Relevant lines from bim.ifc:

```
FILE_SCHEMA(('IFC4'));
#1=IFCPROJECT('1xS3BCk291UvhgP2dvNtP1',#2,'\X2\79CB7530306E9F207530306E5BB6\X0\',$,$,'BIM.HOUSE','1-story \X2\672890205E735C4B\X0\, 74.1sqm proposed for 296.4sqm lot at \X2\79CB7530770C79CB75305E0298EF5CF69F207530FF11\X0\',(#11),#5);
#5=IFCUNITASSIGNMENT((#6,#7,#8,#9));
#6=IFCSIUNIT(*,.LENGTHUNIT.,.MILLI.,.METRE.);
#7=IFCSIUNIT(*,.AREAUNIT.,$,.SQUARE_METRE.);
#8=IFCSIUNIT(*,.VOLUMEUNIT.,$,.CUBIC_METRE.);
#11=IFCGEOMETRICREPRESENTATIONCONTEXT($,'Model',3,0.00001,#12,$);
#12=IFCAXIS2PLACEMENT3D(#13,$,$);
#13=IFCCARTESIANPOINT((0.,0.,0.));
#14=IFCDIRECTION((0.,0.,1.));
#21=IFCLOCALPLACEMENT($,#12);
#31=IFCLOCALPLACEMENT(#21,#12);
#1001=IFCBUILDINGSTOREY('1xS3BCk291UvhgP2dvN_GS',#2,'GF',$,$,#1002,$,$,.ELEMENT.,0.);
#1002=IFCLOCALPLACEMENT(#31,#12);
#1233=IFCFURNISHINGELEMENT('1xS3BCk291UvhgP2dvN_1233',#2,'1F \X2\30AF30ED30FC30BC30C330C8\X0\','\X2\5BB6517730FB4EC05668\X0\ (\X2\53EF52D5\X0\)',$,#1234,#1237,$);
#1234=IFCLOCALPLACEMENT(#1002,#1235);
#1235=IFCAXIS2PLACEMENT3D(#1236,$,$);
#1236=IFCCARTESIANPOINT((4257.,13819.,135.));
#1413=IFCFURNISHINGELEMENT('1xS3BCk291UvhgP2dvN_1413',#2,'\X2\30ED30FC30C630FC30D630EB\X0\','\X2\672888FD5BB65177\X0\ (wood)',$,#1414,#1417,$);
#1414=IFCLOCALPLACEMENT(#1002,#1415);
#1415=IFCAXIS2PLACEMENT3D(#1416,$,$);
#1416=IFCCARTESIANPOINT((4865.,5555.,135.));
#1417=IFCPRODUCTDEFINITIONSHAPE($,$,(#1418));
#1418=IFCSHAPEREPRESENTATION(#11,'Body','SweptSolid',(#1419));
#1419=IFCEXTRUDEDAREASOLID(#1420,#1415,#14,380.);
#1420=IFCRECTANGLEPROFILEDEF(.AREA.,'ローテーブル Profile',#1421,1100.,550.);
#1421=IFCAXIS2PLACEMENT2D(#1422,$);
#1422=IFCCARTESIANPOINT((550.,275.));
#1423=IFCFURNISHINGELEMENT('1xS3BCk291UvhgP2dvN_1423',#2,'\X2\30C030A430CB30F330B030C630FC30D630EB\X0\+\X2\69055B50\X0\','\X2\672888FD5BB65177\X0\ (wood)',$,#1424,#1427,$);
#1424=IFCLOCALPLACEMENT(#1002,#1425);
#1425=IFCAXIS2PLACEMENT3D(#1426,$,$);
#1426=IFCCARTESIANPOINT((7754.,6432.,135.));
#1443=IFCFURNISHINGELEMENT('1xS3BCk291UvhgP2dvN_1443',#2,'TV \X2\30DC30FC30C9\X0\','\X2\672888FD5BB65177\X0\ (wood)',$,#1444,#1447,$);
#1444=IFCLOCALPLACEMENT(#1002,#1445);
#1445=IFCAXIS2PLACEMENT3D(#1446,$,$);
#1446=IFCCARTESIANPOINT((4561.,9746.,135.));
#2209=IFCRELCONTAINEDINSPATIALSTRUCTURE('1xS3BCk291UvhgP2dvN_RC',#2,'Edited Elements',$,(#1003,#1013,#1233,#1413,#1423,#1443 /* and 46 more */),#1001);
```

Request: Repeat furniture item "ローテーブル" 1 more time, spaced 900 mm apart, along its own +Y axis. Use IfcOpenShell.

```python
import ifcopenshell
import ifcopenshell.api.geometry
import ifcopenshell.api.root
import ifcopenshell.util.element
import ifcopenshell.util.placement
import ifcopenshell.util.unit

model = ifcopenshell.open("bim.ifc")
unit_scale = ifcopenshell.util.unit.calculate_unit_scale(model)


def reuse_history(source, copy):
    """copy_class also copies each property set's owner history, people and application; keep the originals."""
    for rel in copy.IsDefinedBy:
        if rel.is_a("IfcRelDefinesByProperties") and (history := rel.RelatingPropertyDefinition.OwnerHistory):
            rel.RelatingPropertyDefinition.OwnerHistory = source.OwnerHistory
            ifcopenshell.util.element.remove_deep2(model, history)


source = model.by_guid("1xS3BCk291UvhgP2dvN_1413")
base = ifcopenshell.util.placement.get_local_placement(source.ObjectPlacement)
step = base[:3, 1] * 0.9 / unit_scale

for i in range(1, 2):
    copy = ifcopenshell.api.root.copy_class(model, product=source)
    copy.Representation = ifcopenshell.util.element.copy_deep(
        model, source.Representation, exclude=["IfcGeometricRepresentationContext", "IfcRepresentationMap"]
    )
    reuse_history(source, copy)
    matrix = base.copy()
    matrix[:3, 3] += i * step
    print("added at", matrix[:3, 3].round(3) + 0.0)
    ifcopenshell.api.geometry.edit_object_placement(model, product=copy, matrix=matrix, is_si=False)

model.write("bim_v2.ifc")
```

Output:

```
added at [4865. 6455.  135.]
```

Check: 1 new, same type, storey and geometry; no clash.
